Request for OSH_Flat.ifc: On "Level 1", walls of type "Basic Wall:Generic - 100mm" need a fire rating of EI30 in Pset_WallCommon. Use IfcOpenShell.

First a look at what the model holds.

```python
import ifcopenshell
import ifcopenshell.util.element

model = ifcopenshell.open("OSH_Flat.ifc")
print(model.schema)
storey = next(s for s in model.by_type("IfcBuildingStorey") if s.Name == "Level 1")
walls = [e for e in ifcopenshell.util.element.get_decomposition(storey) if e.is_a("IfcWall")]
seen = {}
for e in walls:
    element_type = ifcopenshell.util.element.get_type(e)
    key = (element_type.Name if element_type != e and element_type else None, ifcopenshell.util.element.get_pset(e, "Pset_WallCommon", "FireRating"))
    seen[key] = seen.get(key, 0) + 1
for (name, value), count in sorted(seen.items(), key=str):
    print(count, "x", name, "|", value)
```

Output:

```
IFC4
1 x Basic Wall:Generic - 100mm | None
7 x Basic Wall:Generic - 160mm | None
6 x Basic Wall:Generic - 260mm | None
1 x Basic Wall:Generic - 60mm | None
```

```python
import ifcopenshell
import ifcopenshell.api.pset
import ifcopenshell.util.element

model = ifcopenshell.open("OSH_Flat.ifc")

storey = next(s for s in model.by_type("IfcBuildingStorey") if s.Name == "Level 1")
walls = [e for e in ifcopenshell.util.element.get_decomposition(storey) if e.is_a("IfcWall")]

count = 0
for e in walls:
    element_type = ifcopenshell.util.element.get_type(e)
    if element_type in (None, e) or element_type.Name != "Basic Wall:Generic - 100mm":
        continue
    # add_pset returns the element's existing set when there is one.
    pset = ifcopenshell.api.pset.add_pset(model, product=e, name="Pset_WallCommon")
    ifcopenshell.api.pset.edit_pset(model, pset=pset, properties={"FireRating": "EI30"})
    count += 1

print(count, "walls updated")

model.write("OSH_Flat_v2.ifc")
```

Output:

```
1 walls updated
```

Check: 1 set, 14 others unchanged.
